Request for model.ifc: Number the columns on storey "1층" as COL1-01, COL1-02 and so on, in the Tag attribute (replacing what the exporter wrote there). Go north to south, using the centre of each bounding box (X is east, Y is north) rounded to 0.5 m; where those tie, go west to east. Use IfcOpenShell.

First a look at what the model holds.

```python
import ifcopenshell
import ifcopenshell.util.element
import ifcopenshell.util.placement

model = ifcopenshell.open("model.ifc")
print(model.schema)
storey = next(s for s in model.by_type("IfcBuildingStorey") if s.Name == "1층")
columns = [e for e in ifcopenshell.util.element.get_decomposition(storey) if e.is_a("IfcColumn")]
for e in sorted(columns, key=lambda e: e.id()):
    origin = ifcopenshell.util.placement.get_local_placement(e.ObjectPlacement)[:3, 3]
    print(e.id(), e.Tag, e.Name, origin.round(2) + 0.0, sep=" | ")
```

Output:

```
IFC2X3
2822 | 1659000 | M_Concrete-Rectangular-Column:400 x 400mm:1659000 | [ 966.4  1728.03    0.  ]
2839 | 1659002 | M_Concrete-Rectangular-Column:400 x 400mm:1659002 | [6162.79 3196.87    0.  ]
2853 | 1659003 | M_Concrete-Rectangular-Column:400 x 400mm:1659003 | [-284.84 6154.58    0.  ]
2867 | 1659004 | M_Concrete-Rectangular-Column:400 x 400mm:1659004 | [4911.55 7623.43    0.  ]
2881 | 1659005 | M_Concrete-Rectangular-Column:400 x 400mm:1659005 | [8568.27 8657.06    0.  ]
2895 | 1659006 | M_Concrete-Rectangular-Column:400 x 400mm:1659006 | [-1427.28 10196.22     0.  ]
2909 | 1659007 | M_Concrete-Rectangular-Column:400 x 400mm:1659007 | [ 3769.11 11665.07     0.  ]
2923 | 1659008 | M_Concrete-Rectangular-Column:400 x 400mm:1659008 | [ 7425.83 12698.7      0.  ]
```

```python
import ifcopenshell
import ifcopenshell.geom
import ifcopenshell.util.element
import ifcopenshell.util.shape

model = ifcopenshell.open("model.ifc")
settings = ifcopenshell.geom.settings()
settings.set("use-world-coords", True)


def centre(element):
    shape = ifcopenshell.geom.create_shape(settings, element)
    return ifcopenshell.util.shape.get_bbox_centroid(shape.geometry)


storey = next(s for s in model.by_type("IfcBuildingStorey") if s.Name == "1층")
columns = [e for e in ifcopenshell.util.element.get_decomposition(storey) if e.is_a("IfcColumn")]

# Insertion points can sit at a corner or the storey origin, so sort by the geometry (in metres).
centres = {e: centre(e) for e in columns}
columns.sort(key=lambda e: (-round(centres[e][1] / 0.5), centres[e][0]))

for i, e in enumerate(columns, start=1):
    number = f"COL1-{i:02d}"
    e.Tag = number
    print(e.id(), number)

model.write("model_updated.ifc")
```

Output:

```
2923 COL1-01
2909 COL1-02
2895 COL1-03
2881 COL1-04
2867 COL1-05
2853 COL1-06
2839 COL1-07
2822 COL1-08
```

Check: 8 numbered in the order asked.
